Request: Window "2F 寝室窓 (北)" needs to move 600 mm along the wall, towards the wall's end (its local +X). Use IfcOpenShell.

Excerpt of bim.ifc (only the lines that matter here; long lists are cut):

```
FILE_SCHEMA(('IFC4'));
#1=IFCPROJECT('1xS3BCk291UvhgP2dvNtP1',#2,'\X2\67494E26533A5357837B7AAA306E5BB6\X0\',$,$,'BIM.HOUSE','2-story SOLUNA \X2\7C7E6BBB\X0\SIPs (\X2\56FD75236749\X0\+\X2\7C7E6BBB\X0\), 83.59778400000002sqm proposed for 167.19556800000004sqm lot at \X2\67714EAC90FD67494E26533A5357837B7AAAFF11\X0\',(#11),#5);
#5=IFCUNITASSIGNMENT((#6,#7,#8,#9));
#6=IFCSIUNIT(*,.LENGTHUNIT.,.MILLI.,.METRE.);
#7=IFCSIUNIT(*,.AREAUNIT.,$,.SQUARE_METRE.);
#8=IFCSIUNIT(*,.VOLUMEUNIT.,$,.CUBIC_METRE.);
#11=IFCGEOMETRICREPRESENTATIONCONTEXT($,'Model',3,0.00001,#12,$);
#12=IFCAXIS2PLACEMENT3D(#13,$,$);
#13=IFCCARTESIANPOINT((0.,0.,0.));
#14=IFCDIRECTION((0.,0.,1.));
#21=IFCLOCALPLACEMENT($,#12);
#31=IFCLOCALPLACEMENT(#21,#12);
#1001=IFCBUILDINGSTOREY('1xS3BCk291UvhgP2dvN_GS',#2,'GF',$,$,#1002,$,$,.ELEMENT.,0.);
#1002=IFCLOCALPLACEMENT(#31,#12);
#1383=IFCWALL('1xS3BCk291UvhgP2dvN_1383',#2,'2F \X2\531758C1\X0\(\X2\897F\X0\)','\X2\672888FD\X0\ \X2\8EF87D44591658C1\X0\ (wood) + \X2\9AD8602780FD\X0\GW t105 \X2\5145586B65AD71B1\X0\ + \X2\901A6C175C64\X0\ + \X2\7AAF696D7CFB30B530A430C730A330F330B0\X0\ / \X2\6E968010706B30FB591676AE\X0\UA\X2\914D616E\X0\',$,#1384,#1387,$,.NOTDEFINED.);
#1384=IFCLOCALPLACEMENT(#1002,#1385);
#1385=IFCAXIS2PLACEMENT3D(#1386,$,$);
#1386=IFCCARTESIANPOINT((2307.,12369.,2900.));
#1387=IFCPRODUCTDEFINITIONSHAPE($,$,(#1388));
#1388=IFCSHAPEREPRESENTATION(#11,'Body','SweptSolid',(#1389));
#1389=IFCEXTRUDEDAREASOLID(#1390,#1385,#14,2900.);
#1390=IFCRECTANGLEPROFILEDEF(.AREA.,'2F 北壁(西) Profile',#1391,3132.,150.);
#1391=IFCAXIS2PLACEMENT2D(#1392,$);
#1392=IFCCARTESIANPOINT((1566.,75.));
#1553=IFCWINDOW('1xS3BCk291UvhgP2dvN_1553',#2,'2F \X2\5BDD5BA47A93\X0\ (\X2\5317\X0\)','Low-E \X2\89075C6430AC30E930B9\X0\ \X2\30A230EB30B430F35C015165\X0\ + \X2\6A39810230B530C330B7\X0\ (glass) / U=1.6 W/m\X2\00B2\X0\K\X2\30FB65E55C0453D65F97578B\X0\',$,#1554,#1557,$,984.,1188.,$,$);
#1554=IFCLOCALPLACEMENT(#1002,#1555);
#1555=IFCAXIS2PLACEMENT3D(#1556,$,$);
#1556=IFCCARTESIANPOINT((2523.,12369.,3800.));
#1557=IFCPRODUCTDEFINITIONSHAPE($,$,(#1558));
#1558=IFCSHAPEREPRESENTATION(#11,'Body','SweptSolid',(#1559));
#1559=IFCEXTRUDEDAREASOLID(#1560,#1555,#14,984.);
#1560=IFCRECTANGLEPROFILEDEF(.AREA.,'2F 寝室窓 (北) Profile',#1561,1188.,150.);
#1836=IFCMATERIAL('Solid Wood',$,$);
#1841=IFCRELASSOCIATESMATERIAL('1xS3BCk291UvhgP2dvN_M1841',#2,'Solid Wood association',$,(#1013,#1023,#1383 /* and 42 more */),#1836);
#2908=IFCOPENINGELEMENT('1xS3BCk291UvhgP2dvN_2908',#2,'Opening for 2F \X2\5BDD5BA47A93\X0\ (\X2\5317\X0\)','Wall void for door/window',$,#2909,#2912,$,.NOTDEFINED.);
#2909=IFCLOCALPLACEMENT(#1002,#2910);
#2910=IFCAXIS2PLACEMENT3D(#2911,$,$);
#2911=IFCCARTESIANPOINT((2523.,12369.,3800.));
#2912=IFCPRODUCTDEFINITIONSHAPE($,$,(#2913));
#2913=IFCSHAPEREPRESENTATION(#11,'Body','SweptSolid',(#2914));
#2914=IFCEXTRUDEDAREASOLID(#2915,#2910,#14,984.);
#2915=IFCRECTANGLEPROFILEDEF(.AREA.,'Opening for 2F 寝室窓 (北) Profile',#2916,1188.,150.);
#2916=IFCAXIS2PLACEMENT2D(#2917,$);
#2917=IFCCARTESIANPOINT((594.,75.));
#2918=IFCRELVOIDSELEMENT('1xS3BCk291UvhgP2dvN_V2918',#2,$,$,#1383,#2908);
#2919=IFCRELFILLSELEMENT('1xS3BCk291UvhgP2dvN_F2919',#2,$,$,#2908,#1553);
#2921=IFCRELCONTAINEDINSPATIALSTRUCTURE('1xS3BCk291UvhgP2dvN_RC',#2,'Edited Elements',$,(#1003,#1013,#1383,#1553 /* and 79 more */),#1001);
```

```python
import ifcopenshell
import ifcopenshell.api.geometry
import ifcopenshell.util.placement

model = ifcopenshell.open("bim.ifc")

window = model.by_guid("1xS3BCk291UvhgP2dvN_1553")
opening = window.FillsVoids[0].RelatingOpeningElement
wall = opening.VoidsElements[0].RelatingBuildingElement

wall_matrix = ifcopenshell.util.placement.get_local_placement(wall.ObjectPlacement)
shift = wall_matrix[:3, 0] * 600.0
before = ifcopenshell.util.placement.get_local_placement(window.ObjectPlacement)[:3, 3].copy()

# The window is not placed relative to its opening, so move both.
for product in (opening, window):
    matrix = ifcopenshell.util.placement.get_local_placement(product.ObjectPlacement)
    matrix[:3, 3] += shift
    ifcopenshell.api.geometry.edit_object_placement(model, product=product, matrix=matrix, is_si=False)

after = ifcopenshell.util.placement.get_local_placement(window.ObjectPlacement)[:3, 3]
print("window moved by", (after - before).round(3) + 0.0)

model.write("bim_rev.ifc")
```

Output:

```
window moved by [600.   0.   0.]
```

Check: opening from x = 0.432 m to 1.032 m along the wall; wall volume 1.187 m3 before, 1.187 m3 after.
